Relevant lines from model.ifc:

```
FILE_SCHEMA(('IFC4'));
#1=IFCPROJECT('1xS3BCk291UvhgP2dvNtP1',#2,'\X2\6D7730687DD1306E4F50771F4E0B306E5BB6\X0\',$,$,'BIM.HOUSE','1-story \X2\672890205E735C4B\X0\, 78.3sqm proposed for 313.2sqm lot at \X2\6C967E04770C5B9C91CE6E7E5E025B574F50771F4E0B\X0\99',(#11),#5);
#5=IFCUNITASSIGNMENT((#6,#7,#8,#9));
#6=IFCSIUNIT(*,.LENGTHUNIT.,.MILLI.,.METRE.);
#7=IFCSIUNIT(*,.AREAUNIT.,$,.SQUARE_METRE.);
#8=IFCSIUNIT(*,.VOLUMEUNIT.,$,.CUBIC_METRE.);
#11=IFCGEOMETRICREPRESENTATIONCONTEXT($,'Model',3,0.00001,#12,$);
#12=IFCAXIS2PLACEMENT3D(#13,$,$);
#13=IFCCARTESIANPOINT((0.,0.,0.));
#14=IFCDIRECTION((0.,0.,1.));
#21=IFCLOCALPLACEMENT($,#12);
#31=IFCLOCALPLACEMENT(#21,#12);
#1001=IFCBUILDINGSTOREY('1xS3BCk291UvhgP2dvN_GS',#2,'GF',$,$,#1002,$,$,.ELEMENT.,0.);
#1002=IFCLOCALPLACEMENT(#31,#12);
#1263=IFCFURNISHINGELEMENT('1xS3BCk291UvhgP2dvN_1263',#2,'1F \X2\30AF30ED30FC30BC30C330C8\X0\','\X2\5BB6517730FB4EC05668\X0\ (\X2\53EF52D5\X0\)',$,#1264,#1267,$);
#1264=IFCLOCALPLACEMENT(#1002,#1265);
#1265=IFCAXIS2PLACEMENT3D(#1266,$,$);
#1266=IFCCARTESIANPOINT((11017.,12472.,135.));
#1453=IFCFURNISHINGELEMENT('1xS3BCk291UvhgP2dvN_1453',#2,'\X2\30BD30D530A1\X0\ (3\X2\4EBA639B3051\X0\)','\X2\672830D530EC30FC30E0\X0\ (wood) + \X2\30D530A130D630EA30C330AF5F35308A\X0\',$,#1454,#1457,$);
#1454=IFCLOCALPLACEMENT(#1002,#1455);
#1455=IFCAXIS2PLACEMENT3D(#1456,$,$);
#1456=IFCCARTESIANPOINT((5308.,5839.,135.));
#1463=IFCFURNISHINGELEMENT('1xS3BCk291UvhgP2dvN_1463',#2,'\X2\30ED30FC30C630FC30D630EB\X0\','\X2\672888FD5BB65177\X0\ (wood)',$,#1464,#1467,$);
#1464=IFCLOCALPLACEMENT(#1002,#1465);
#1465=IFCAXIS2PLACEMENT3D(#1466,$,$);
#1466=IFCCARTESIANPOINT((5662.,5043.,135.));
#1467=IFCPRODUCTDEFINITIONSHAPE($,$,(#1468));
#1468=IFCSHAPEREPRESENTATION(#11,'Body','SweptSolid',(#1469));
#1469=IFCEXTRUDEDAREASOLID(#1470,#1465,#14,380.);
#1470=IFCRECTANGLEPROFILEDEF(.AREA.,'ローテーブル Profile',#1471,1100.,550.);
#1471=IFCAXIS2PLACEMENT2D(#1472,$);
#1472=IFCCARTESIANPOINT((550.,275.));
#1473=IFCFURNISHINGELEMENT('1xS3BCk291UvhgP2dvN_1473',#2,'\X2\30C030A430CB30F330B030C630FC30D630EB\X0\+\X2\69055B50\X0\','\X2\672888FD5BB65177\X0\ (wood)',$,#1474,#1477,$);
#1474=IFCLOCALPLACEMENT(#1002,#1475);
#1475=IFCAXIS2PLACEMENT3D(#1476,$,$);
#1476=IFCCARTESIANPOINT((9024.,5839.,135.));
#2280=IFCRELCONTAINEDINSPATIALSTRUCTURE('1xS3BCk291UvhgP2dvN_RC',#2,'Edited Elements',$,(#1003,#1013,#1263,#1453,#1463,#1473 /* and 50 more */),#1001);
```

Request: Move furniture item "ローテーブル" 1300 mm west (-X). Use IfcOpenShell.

```python
import ifcopenshell
import ifcopenshell.api.geometry
import ifcopenshell.util.placement

model = ifcopenshell.open("model.ifc")

item = model.by_guid("1xS3BCk291UvhgP2dvN_1463")
matrix = ifcopenshell.util.placement.get_local_placement(item.ObjectPlacement)
matrix[0, 3] -= 1300.0
ifcopenshell.api.geometry.edit_object_placement(model, product=item, matrix=matrix, is_si=False)

print(ifcopenshell.util.placement.get_local_placement(item.ObjectPlacement).round(3) + 0.0)

model.write("model_edited.ifc")
```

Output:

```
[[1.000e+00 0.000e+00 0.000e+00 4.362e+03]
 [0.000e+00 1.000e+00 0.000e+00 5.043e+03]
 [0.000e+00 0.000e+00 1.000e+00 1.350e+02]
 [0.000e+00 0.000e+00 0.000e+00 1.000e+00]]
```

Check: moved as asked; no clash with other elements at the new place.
